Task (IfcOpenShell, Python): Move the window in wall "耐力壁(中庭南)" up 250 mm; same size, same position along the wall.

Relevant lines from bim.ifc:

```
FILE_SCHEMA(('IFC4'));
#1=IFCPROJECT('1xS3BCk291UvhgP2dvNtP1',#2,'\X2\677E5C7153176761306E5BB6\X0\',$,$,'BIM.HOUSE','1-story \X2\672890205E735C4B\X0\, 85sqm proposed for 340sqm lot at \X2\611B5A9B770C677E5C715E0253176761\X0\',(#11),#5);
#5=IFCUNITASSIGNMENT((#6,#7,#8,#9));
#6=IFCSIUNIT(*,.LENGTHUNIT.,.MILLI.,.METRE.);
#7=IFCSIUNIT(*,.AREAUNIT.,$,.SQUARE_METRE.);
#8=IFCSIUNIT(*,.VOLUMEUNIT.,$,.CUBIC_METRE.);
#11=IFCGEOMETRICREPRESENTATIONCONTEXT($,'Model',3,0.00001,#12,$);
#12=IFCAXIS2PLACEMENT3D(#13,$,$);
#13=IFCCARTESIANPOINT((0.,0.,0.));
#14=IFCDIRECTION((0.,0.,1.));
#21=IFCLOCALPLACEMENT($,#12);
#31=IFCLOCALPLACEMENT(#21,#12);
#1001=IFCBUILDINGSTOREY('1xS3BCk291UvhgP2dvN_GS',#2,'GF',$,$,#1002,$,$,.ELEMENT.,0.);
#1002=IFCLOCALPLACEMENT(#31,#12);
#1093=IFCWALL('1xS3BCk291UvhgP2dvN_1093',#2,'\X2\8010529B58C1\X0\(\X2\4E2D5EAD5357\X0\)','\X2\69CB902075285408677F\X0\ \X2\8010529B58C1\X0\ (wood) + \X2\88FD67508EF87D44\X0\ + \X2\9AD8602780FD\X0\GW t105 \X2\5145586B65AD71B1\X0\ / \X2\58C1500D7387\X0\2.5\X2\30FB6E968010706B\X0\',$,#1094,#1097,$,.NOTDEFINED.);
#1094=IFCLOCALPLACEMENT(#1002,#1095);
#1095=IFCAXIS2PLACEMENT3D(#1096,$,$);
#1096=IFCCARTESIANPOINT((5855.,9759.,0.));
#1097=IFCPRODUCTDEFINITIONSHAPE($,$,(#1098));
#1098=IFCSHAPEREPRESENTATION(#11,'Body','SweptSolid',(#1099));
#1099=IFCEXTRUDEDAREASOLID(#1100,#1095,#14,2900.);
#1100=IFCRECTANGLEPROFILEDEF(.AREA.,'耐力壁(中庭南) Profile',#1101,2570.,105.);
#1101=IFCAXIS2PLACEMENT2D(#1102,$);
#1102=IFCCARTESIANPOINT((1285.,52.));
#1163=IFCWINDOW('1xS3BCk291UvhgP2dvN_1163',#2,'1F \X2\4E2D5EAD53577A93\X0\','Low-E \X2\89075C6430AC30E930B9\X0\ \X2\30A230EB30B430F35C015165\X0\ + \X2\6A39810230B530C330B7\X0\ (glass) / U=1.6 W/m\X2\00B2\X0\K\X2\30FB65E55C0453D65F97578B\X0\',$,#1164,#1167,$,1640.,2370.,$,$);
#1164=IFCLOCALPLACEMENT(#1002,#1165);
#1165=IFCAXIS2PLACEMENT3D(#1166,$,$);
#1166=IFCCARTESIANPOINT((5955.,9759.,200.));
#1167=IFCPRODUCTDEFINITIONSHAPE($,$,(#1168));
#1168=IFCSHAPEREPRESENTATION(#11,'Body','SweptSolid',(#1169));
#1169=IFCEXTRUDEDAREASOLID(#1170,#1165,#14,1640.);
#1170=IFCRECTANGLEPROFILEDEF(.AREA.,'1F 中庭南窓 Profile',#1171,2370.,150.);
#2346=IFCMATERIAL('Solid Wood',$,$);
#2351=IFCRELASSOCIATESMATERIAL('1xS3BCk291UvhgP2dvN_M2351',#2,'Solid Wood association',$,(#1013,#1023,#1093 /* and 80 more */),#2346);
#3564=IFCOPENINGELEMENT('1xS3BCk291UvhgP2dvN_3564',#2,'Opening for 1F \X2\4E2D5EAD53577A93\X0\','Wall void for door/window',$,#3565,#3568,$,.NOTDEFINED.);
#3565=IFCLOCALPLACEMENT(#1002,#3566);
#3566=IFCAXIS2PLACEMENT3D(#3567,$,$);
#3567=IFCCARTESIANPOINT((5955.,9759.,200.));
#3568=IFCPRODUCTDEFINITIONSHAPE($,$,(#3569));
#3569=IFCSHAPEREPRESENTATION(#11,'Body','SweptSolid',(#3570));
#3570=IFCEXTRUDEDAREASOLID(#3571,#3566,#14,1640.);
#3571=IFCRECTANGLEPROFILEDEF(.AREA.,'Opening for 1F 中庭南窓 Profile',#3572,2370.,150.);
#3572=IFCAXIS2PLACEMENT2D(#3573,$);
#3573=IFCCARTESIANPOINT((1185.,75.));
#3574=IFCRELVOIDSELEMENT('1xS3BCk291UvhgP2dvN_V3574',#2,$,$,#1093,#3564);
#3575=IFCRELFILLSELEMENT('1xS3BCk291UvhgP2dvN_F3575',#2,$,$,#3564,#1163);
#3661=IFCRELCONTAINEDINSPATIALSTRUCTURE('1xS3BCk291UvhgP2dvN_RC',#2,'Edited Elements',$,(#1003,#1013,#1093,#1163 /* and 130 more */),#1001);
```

```python
import numpy as np
import ifcopenshell
import ifcopenshell.api.geometry
import ifcopenshell.util.placement
import ifcopenshell.util.unit

model = ifcopenshell.open("bim.ifc")
unit_scale = ifcopenshell.util.unit.calculate_unit_scale(model)

window = model.by_guid("1xS3BCk291UvhgP2dvN_1163")
opening = window.FillsVoids[0].RelatingOpeningElement
dz = 0.25 / unit_scale

shift = np.array([0.0, 0.0, dz])
# The window is not placed relative to its opening, so move both.
for product in (opening, window):
    matrix = ifcopenshell.util.placement.get_local_placement(product.ObjectPlacement)
    matrix[:3, 3] += shift
    ifcopenshell.api.geometry.edit_object_placement(model, product=product, matrix=matrix, is_si=False)

print(f"moved by {dz * unit_scale:+.3f} m")

model.write("bim_rev.ifc")
```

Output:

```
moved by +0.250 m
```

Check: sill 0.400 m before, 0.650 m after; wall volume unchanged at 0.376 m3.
